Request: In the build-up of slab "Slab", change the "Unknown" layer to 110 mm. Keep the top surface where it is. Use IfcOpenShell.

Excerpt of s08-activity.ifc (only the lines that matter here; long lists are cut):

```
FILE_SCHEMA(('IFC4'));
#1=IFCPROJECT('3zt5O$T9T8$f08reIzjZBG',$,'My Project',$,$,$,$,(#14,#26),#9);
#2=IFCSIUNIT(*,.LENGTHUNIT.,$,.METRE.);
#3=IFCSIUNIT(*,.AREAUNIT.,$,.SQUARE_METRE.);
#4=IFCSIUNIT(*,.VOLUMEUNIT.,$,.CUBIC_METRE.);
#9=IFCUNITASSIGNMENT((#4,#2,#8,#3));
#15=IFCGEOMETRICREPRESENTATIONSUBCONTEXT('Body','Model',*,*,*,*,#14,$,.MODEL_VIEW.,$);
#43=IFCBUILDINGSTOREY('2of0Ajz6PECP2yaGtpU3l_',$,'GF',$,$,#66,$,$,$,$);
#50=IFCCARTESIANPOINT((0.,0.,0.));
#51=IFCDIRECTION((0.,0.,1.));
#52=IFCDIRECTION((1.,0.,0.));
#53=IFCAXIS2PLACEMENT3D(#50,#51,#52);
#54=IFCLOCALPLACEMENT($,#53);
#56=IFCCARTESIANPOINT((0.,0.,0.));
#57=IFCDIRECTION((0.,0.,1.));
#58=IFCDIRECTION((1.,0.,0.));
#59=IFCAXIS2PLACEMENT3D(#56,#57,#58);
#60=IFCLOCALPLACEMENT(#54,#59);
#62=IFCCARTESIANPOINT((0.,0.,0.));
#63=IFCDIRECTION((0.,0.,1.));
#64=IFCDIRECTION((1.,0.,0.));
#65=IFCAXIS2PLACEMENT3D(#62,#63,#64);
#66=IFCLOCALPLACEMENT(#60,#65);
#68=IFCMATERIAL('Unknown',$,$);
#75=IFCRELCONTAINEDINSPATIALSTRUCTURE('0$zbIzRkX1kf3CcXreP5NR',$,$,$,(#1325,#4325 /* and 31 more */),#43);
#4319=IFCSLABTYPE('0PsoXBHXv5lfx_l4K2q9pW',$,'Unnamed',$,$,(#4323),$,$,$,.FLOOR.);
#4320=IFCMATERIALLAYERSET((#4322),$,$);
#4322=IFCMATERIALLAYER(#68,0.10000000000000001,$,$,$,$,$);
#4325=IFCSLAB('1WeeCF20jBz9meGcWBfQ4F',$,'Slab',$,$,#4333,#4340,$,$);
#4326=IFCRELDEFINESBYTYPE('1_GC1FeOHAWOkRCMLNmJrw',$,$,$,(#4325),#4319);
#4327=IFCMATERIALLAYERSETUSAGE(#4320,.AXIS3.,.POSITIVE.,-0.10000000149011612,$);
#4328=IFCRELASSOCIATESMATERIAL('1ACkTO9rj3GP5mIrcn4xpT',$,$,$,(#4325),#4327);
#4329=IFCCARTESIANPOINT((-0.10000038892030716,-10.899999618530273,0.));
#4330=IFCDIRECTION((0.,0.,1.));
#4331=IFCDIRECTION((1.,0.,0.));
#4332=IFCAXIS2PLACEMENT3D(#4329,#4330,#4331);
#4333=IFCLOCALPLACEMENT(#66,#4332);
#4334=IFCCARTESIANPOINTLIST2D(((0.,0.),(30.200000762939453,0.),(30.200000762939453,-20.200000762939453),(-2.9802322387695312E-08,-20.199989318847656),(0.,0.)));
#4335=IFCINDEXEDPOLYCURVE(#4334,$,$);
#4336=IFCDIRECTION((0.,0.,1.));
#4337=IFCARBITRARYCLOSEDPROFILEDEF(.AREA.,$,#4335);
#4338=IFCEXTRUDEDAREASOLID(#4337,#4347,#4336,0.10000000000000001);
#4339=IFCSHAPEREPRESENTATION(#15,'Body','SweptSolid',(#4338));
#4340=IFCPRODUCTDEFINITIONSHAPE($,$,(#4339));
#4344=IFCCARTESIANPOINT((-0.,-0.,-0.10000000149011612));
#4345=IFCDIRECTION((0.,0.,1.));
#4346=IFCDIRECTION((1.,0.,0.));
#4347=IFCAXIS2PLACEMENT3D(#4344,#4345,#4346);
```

```python
import ifcopenshell
import ifcopenshell.util.element
import ifcopenshell.util.representation

model = ifcopenshell.open("s08-activity.ifc")

layer_set = model.by_id(4320)
layer = next(l for l in layer_set.MaterialLayers if l.Material and l.Material.Name == "Unknown")
change = 0.11 - layer.LayerThickness
layer.LayerThickness += change

# Geometry does not follow the layer set by itself.
slabs = [e for e in ifcopenshell.util.element.get_elements_by_material(model, layer_set) if e.is_a("IfcSlab")]
for slab in sorted(slabs, key=lambda e: e.id()):
    body = ifcopenshell.util.representation.get_representation(slab, "Model", "Body")
    solid = body.Items[0]
    old_depth = solid.Depth
    solid.Depth += change
    # Extruded upwards: lower the start of the extrusion so the top stays.
    x, y, z = solid.Position.Location.Coordinates
    solid.Position.Location = model.createIfcCartesianPoint((x, y, z - change))
    print(slab.id(), f"{old_depth:g} -> {solid.Depth:g}")

# The layers are counted up from the underside, which has moved.
for usage in {ifcopenshell.util.element.get_material(slab) for slab in slabs}:
    usage.OffsetFromReferenceLine -= change

model.write("s08-activity_rev.ifc")
```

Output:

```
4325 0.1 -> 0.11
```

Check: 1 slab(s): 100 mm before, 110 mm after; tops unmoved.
